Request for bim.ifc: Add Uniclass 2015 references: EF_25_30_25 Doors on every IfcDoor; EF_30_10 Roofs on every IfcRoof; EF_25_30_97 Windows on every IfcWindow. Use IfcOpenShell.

First a look at what the model holds.

```python
import ifcopenshell

model = ifcopenshell.open("bim.ifc")
print(model.schema)
print("classifications:", [c.Name for c in model.by_type("IfcClassification")])
for ifc_class in ("IfcDoor", "IfcRoof", "IfcStair", "IfcWall", "IfcWindow"):
    print(ifc_class, len(model.by_type(ifc_class)))
```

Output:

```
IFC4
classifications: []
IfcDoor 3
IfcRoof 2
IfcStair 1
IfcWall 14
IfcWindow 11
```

```python
import ifcopenshell
import ifcopenshell.api.classification

model = ifcopenshell.open("bim.ifc")

system = ifcopenshell.api.classification.add_classification(model, classification="Uniclass 2015")

codes = {
    "IfcDoor": ("EF_25_30_25", "Doors"),
    "IfcRoof": ("EF_30_10", "Roofs"),
    "IfcWindow": ("EF_25_30_97", "Windows"),
}
for ifc_class, (code, name) in codes.items():
    products = model.by_type(ifc_class)
    ifcopenshell.api.classification.add_reference(
        model, products=products, classification=system, identification=code, name=name
    )
    print(code, len(products))

model.write("bim_rev.ifc")
```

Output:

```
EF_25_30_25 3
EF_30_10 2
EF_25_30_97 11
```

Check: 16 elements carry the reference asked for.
